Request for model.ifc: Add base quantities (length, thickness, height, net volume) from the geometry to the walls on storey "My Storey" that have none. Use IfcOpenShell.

First a look at what the model holds.

```python
import ifcopenshell
import ifcopenshell.util.element
import ifcopenshell.util.unit

model = ifcopenshell.open("model.ifc")
print(model.schema)
for unit_type in ("LENGTHUNIT", "AREAUNIT", "VOLUMEUNIT"):
    print(unit_type, ifcopenshell.util.unit.calculate_unit_scale(model, unit_type))
storey = next(s for s in model.by_type("IfcBuildingStorey") if s.Name == "My Storey")
walls = [e for e in ifcopenshell.util.element.get_decomposition(storey) if e.is_a("IfcWall")]
for e in sorted(walls, key=lambda e: e.id()):
    print(e.id(), e.is_a(), e.Name, list(ifcopenshell.util.element.get_psets(e, qtos_only=True)), sep=" | ")
```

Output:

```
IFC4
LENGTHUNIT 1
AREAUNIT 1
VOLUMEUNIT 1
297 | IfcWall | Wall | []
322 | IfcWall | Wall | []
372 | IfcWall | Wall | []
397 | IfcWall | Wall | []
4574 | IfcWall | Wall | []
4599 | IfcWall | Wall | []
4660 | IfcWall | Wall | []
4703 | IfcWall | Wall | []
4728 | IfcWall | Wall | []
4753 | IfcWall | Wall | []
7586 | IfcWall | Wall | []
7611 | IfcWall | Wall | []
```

```python
import ifcopenshell
import ifcopenshell.api.pset
import ifcopenshell.geom
import ifcopenshell.util.element
import ifcopenshell.util.shape
import ifcopenshell.util.unit

model = ifcopenshell.open("model.ifc")
unit_scale = ifcopenshell.util.unit.calculate_unit_scale(model)
volume_scale = ifcopenshell.util.unit.calculate_unit_scale(model, "VOLUMEUNIT")
settings = ifcopenshell.geom.settings()

storey = next(s for s in model.by_type("IfcBuildingStorey") if s.Name == "My Storey")
walls = [e for e in ifcopenshell.util.element.get_decomposition(storey) if e.is_a("IfcWall")]

for e in sorted(walls, key=lambda e: e.id()):
    if ifcopenshell.util.element.get_psets(e, qtos_only=True, should_inherit=False):
        continue
    # Geometry comes back in metres, in the element's own axes.
    shape = ifcopenshell.geom.create_shape(settings, e)
    values = {
        "Length": ifcopenshell.util.shape.get_x(shape.geometry) / unit_scale,
        "Width": ifcopenshell.util.shape.get_y(shape.geometry) / unit_scale,
        "Height": ifcopenshell.util.shape.get_z(shape.geometry) / unit_scale,
        "NetVolume": ifcopenshell.util.shape.get_volume(shape.geometry) / volume_scale,
    }
    qto = ifcopenshell.api.pset.add_qto(model, product=e, name="Qto_WallBaseQuantities")
    ifcopenshell.api.pset.edit_qto(model, qto=qto, properties=values)
    print(e.id(), {k: round(v, 3) for k, v in values.items()})

model.write("model_v2.ifc")
```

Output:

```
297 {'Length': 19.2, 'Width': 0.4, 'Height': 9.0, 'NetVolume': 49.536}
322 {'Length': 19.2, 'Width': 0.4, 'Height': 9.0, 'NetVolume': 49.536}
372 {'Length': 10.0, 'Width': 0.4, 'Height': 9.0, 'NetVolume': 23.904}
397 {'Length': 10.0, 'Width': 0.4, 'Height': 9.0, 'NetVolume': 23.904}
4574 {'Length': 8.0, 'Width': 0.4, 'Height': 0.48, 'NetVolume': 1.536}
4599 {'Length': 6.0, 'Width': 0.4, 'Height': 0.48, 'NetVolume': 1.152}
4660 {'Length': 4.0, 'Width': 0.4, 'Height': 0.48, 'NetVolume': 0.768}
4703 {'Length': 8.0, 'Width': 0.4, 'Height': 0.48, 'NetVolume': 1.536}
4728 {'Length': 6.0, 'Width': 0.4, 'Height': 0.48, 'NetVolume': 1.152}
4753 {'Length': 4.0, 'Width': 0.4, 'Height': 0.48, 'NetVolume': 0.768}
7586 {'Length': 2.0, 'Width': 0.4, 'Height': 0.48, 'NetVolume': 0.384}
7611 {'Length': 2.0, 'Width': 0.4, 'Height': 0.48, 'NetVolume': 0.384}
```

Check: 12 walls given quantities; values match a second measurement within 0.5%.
